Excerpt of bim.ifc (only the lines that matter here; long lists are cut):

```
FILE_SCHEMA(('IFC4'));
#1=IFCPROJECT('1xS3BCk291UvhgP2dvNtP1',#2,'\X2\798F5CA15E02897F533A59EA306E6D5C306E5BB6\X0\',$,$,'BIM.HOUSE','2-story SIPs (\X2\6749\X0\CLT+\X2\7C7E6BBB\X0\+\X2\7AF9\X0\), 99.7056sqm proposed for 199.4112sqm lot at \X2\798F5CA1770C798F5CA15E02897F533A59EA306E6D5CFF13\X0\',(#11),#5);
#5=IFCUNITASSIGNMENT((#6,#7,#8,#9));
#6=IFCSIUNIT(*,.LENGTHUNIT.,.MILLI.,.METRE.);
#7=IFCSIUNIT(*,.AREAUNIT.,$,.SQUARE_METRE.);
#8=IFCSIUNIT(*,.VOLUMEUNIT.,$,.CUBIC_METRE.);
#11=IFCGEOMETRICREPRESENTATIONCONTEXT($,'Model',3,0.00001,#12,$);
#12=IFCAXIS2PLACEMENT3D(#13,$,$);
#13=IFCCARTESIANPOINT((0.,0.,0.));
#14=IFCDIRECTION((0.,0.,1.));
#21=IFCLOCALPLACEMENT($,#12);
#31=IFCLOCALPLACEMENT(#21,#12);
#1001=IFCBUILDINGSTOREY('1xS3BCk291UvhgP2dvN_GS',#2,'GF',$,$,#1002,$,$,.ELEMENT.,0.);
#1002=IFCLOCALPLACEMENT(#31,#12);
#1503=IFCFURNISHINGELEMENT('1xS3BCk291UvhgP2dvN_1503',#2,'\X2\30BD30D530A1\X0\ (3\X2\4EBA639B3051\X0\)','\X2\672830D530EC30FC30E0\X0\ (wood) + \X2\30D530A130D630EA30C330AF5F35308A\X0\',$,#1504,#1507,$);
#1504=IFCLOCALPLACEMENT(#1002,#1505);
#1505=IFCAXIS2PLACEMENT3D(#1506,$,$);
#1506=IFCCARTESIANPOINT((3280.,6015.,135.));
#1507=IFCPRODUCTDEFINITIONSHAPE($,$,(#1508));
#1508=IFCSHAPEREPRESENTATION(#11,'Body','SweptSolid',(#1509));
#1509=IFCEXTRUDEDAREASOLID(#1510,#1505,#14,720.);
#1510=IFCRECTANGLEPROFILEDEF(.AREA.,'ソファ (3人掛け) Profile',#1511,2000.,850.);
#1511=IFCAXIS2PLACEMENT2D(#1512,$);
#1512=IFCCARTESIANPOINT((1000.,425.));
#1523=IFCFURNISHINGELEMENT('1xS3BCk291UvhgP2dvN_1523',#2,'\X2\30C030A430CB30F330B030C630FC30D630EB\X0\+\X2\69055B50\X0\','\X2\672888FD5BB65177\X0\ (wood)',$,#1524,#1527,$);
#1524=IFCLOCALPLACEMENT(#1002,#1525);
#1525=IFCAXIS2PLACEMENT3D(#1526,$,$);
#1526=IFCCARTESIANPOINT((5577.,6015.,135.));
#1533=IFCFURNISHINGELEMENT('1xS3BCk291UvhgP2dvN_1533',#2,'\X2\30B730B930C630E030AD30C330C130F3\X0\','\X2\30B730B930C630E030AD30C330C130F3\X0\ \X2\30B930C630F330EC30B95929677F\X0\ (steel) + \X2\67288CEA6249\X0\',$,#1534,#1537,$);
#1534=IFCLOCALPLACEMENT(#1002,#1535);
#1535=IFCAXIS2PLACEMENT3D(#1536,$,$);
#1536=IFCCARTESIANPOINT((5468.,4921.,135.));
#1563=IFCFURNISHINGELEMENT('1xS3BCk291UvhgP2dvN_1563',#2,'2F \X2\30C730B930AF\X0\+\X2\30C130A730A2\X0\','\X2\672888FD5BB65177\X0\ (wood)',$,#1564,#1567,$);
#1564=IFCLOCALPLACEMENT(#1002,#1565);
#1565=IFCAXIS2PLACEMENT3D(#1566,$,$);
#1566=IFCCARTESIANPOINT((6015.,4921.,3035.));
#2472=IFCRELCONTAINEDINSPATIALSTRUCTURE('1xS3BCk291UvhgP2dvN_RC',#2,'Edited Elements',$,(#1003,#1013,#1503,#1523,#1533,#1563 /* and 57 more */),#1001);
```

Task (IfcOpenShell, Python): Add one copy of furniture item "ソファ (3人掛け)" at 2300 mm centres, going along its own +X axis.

```python
import ifcopenshell
import ifcopenshell.api.geometry
import ifcopenshell.api.root
import ifcopenshell.util.element
import ifcopenshell.util.placement
import ifcopenshell.util.unit

model = ifcopenshell.open("bim.ifc")
unit_scale = ifcopenshell.util.unit.calculate_unit_scale(model)


def reuse_history(source, copy):
    """copy_class also copies each property set's owner history, people and application; keep the originals."""
    for rel in copy.IsDefinedBy:
        if rel.is_a("IfcRelDefinesByProperties") and (history := rel.RelatingPropertyDefinition.OwnerHistory):
            rel.RelatingPropertyDefinition.OwnerHistory = source.OwnerHistory
            ifcopenshell.util.element.remove_deep2(model, history)


source = model.by_guid("1xS3BCk291UvhgP2dvN_1503")
base = ifcopenshell.util.placement.get_local_placement(source.ObjectPlacement)
step = base[:3, 0] * 2.3 / unit_scale

for i in range(1, 2):
    copy = ifcopenshell.api.root.copy_class(model, product=source)
    copy.Representation = ifcopenshell.util.element.copy_deep(
        model, source.Representation, exclude=["IfcGeometricRepresentationContext", "IfcRepresentationMap"]
    )
    reuse_history(source, copy)
    matrix = base.copy()
    matrix[:3, 3] += i * step
    print("added at", matrix[:3, 3].round(3) + 0.0)
    ifcopenshell.api.geometry.edit_object_placement(model, product=copy, matrix=matrix, is_si=False)

model.write("bim_rev.ifc")
```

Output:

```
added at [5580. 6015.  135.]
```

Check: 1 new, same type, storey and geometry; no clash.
